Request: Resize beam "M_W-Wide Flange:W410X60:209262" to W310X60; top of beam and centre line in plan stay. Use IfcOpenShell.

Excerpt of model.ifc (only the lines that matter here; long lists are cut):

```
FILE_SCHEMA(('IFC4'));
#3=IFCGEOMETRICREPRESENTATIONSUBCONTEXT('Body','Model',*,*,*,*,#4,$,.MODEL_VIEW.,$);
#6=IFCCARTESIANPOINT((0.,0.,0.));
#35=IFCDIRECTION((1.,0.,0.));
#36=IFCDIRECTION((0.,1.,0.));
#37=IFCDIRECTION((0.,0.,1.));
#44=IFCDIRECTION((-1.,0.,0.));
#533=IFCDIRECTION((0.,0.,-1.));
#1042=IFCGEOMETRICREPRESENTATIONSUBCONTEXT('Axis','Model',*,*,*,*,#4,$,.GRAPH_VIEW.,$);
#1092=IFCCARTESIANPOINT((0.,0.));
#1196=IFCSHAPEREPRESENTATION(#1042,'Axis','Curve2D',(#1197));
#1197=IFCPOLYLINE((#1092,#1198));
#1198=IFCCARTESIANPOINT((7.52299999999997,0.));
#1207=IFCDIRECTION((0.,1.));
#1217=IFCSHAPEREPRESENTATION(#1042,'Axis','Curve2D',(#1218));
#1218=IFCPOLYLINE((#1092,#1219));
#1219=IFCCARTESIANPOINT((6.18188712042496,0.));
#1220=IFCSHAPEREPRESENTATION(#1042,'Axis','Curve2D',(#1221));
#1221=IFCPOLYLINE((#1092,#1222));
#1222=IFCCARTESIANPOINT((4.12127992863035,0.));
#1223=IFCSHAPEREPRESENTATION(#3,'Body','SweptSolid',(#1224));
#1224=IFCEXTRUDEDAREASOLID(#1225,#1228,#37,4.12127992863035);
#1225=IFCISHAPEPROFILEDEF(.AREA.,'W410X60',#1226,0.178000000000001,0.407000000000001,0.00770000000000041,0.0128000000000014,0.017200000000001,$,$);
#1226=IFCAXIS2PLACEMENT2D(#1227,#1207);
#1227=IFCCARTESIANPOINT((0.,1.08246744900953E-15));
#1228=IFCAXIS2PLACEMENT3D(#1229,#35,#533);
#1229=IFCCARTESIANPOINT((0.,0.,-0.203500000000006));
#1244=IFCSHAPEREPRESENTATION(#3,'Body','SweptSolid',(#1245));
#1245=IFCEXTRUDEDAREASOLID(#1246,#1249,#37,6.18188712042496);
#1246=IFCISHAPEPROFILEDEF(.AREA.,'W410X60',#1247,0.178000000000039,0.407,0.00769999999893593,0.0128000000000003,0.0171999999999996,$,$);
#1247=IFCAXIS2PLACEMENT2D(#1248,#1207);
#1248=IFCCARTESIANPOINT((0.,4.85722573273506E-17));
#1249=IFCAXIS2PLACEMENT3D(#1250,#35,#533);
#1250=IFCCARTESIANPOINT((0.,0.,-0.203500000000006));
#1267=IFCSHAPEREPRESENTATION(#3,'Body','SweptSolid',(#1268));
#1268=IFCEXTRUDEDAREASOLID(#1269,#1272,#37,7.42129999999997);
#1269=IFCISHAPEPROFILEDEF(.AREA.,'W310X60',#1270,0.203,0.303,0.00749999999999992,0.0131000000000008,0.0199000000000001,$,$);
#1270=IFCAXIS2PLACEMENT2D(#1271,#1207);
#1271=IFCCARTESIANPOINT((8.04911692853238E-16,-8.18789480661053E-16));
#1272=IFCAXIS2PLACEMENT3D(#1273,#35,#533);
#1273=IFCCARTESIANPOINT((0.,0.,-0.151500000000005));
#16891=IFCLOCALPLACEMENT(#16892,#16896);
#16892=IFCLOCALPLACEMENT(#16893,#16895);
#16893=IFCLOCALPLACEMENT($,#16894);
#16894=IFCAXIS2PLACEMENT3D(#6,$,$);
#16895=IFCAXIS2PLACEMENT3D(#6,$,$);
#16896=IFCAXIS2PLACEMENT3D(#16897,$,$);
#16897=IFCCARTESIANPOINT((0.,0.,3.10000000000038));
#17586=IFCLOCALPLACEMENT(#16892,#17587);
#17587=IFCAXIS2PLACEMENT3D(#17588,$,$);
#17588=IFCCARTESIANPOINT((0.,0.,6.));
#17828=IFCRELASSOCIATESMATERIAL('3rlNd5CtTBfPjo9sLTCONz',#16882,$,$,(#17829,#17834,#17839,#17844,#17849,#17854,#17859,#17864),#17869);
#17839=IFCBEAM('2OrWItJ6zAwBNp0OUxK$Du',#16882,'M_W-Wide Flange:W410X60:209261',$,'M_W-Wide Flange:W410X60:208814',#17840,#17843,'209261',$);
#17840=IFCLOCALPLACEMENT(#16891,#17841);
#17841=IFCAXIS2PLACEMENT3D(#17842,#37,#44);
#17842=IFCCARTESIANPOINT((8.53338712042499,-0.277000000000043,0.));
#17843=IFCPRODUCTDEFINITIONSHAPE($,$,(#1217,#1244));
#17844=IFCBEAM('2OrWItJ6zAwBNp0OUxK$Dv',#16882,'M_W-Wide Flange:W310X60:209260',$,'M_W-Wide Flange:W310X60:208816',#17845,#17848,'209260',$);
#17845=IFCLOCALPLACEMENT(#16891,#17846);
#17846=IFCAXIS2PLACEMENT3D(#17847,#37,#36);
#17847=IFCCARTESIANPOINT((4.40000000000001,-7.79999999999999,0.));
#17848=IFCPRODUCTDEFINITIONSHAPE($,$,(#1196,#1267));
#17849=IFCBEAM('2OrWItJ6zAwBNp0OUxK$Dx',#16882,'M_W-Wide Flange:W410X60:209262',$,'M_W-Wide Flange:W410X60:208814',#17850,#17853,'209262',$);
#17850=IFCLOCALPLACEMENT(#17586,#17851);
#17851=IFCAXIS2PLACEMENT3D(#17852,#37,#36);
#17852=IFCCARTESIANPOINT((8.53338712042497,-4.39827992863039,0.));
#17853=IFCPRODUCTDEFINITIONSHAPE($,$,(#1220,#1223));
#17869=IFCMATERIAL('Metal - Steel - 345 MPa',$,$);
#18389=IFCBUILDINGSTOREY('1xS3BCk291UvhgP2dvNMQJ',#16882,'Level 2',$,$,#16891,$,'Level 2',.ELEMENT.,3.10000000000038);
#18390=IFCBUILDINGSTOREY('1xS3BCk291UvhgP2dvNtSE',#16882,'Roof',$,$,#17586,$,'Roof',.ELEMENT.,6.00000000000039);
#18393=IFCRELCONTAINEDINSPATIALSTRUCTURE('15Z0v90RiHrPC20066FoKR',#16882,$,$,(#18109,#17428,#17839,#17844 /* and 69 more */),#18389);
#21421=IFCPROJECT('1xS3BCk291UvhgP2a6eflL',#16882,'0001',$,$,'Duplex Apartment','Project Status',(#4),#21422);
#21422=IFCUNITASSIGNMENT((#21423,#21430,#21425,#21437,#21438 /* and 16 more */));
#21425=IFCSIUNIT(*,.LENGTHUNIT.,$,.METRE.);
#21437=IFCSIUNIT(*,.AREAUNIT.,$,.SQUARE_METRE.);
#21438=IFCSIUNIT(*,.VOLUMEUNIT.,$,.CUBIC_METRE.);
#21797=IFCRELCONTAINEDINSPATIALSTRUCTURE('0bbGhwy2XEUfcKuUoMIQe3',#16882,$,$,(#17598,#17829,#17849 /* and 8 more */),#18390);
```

```python
import ifcopenshell
import ifcopenshell.util.element
import ifcopenshell.util.representation

model = ifcopenshell.open("model.ifc")

member = model.by_id(17849)
source = next(p for p in model.by_type("IfcIShapeProfileDef") if p.ProfileName == "W310X60")

body = ifcopenshell.util.representation.get_representation(member, "Model", "Body")
solid = body.Items[0]
old_profile = solid.SweptArea

# Copy the section's sizes but keep this member's own profile position.
profile = ifcopenshell.util.element.copy(model, source)
# Profiles are centred, so shift by half the change in depth to hold the top.
shift = (old_profile.OverallDepth - profile.OverallDepth) / 2
x, y = old_profile.Position.Location.Coordinates
up = (-1.0, 0.0)  # upwards, in the solid's own plane
location = model.createIfcCartesianPoint((x + up[0] * shift, y + up[1] * shift))
profile.Position = model.createIfcAxis2Placement2D(location, old_profile.Position.RefDirection)
solid.SweptArea = profile
if not model.get_total_inverses(old_profile):
    ifcopenshell.util.element.remove_deep2(model, old_profile)
member.Name = member.Name.replace("W410X60", "W310X60")
member.ObjectType = member.ObjectType.replace("W410X60", "W310X60")

print(solid.SweptArea)

model.write("model_updated.ifc")
```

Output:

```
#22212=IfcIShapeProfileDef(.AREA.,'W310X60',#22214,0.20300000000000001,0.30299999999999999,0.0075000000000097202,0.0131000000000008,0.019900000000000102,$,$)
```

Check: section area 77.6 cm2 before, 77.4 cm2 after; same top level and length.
